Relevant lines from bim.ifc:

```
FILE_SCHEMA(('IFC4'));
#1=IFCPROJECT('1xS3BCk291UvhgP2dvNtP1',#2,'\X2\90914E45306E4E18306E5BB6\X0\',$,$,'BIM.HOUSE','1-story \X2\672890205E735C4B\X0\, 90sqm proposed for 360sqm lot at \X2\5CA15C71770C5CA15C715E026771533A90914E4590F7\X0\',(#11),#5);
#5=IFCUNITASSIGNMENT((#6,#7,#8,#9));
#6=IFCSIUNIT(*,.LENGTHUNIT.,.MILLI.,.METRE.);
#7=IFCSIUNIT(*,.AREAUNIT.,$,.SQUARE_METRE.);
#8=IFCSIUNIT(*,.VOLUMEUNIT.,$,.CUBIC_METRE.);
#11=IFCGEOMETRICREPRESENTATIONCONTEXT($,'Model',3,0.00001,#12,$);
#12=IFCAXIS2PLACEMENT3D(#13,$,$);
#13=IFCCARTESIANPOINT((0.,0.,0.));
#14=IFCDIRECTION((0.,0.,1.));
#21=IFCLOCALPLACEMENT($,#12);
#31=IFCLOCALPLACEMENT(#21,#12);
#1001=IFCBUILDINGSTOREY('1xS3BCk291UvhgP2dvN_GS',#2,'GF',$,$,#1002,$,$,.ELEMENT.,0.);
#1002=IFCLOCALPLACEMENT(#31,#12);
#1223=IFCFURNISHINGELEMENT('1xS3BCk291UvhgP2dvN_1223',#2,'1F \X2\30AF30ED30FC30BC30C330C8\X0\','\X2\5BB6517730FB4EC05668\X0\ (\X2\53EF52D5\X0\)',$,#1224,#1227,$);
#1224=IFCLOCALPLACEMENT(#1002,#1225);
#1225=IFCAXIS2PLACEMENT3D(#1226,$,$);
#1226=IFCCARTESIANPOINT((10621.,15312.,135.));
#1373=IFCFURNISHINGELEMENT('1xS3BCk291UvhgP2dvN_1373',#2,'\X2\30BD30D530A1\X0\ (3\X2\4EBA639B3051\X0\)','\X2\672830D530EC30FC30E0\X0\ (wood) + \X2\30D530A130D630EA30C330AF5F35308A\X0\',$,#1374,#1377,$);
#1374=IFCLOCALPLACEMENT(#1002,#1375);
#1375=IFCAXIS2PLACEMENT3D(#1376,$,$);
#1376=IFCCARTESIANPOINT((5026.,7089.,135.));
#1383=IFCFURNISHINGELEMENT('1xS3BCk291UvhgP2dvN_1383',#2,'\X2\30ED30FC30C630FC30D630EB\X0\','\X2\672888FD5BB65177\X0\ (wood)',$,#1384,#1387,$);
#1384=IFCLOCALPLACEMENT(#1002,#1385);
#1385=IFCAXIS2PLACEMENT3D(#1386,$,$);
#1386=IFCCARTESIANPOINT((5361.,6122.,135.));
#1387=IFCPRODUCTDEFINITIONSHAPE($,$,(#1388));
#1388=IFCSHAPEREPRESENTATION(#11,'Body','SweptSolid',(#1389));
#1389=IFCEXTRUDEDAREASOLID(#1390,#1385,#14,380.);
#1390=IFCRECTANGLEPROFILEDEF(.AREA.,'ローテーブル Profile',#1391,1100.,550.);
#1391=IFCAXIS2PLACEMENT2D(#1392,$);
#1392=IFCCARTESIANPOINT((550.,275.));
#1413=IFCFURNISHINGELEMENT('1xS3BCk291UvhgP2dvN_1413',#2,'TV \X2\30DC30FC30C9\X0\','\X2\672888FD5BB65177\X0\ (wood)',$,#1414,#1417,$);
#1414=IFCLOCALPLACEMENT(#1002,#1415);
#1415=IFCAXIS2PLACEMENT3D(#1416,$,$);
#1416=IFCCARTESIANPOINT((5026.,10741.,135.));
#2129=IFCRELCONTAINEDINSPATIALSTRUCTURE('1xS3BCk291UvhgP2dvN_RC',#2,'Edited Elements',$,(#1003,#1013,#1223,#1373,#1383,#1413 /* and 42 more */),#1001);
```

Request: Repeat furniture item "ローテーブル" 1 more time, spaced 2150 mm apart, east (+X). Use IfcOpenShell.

```python
import numpy as np
import ifcopenshell
import ifcopenshell.api.geometry
import ifcopenshell.api.root
import ifcopenshell.util.element
import ifcopenshell.util.placement

model = ifcopenshell.open("bim.ifc")


def reuse_history(source, copy):
    """copy_class also copies each property set's owner history, people and application; keep the originals."""
    for rel in copy.IsDefinedBy:
        if rel.is_a("IfcRelDefinesByProperties") and (history := rel.RelatingPropertyDefinition.OwnerHistory):
            rel.RelatingPropertyDefinition.OwnerHistory = source.OwnerHistory
            ifcopenshell.util.element.remove_deep2(model, history)


source = model.by_guid("1xS3BCk291UvhgP2dvN_1383")
base = ifcopenshell.util.placement.get_local_placement(source.ObjectPlacement)
step = np.array([1.0, 0.0, 0.0]) * 2150.0

for i in range(1, 2):
    copy = ifcopenshell.api.root.copy_class(model, product=source)
    copy.Representation = ifcopenshell.util.element.copy_deep(
        model, source.Representation, exclude=["IfcGeometricRepresentationContext", "IfcRepresentationMap"]
    )
    reuse_history(source, copy)
    matrix = base.copy()
    matrix[:3, 3] += i * step
    print("added at", matrix[:3, 3].round(3) + 0.0)
    ifcopenshell.api.geometry.edit_object_placement(model, product=copy, matrix=matrix, is_si=False)

model.write("bim_edited.ifc")
```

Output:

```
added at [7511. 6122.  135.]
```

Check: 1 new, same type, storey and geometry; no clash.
